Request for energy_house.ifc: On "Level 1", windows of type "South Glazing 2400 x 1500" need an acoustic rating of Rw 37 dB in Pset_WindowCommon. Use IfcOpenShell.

First a look at what the model holds.

```python
import ifcopenshell
import ifcopenshell.util.element

model = ifcopenshell.open("energy_house.ifc")
print(model.schema)
storey = next(s for s in model.by_type("IfcBuildingStorey") if s.Name == "Level 1")
windows = [e for e in ifcopenshell.util.element.get_decomposition(storey) if e.is_a("IfcWindow")]
seen = {}
for e in windows:
    element_type = ifcopenshell.util.element.get_type(e)
    key = (element_type.Name if element_type != e and element_type else None, ifcopenshell.util.element.get_pset(e, "Pset_WindowCommon", "AcousticRating"))
    seen[key] = seen.get(key, 0) + 1
for (name, value), count in sorted(seen.items(), key=str):
    print(count, "x", name, "|", value)
```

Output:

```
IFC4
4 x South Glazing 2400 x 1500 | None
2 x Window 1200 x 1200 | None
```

```python
import ifcopenshell
import ifcopenshell.api.pset
import ifcopenshell.util.element

model = ifcopenshell.open("energy_house.ifc")

storey = next(s for s in model.by_type("IfcBuildingStorey") if s.Name == "Level 1")
windows = [e for e in ifcopenshell.util.element.get_decomposition(storey) if e.is_a("IfcWindow")]

count = 0
for e in windows:
    element_type = ifcopenshell.util.element.get_type(e)
    if element_type in (None, e) or element_type.Name != "South Glazing 2400 x 1500":
        continue
    # add_pset returns the element's existing set when there is one.
    pset = ifcopenshell.api.pset.add_pset(model, product=e, name="Pset_WindowCommon")
    ifcopenshell.api.pset.edit_pset(model, pset=pset, properties={"AcousticRating": "Rw 37 dB"})
    count += 1

print(count, "windows updated")

model.write("energy_house_v2.ifc")
```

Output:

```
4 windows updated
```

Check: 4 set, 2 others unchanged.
